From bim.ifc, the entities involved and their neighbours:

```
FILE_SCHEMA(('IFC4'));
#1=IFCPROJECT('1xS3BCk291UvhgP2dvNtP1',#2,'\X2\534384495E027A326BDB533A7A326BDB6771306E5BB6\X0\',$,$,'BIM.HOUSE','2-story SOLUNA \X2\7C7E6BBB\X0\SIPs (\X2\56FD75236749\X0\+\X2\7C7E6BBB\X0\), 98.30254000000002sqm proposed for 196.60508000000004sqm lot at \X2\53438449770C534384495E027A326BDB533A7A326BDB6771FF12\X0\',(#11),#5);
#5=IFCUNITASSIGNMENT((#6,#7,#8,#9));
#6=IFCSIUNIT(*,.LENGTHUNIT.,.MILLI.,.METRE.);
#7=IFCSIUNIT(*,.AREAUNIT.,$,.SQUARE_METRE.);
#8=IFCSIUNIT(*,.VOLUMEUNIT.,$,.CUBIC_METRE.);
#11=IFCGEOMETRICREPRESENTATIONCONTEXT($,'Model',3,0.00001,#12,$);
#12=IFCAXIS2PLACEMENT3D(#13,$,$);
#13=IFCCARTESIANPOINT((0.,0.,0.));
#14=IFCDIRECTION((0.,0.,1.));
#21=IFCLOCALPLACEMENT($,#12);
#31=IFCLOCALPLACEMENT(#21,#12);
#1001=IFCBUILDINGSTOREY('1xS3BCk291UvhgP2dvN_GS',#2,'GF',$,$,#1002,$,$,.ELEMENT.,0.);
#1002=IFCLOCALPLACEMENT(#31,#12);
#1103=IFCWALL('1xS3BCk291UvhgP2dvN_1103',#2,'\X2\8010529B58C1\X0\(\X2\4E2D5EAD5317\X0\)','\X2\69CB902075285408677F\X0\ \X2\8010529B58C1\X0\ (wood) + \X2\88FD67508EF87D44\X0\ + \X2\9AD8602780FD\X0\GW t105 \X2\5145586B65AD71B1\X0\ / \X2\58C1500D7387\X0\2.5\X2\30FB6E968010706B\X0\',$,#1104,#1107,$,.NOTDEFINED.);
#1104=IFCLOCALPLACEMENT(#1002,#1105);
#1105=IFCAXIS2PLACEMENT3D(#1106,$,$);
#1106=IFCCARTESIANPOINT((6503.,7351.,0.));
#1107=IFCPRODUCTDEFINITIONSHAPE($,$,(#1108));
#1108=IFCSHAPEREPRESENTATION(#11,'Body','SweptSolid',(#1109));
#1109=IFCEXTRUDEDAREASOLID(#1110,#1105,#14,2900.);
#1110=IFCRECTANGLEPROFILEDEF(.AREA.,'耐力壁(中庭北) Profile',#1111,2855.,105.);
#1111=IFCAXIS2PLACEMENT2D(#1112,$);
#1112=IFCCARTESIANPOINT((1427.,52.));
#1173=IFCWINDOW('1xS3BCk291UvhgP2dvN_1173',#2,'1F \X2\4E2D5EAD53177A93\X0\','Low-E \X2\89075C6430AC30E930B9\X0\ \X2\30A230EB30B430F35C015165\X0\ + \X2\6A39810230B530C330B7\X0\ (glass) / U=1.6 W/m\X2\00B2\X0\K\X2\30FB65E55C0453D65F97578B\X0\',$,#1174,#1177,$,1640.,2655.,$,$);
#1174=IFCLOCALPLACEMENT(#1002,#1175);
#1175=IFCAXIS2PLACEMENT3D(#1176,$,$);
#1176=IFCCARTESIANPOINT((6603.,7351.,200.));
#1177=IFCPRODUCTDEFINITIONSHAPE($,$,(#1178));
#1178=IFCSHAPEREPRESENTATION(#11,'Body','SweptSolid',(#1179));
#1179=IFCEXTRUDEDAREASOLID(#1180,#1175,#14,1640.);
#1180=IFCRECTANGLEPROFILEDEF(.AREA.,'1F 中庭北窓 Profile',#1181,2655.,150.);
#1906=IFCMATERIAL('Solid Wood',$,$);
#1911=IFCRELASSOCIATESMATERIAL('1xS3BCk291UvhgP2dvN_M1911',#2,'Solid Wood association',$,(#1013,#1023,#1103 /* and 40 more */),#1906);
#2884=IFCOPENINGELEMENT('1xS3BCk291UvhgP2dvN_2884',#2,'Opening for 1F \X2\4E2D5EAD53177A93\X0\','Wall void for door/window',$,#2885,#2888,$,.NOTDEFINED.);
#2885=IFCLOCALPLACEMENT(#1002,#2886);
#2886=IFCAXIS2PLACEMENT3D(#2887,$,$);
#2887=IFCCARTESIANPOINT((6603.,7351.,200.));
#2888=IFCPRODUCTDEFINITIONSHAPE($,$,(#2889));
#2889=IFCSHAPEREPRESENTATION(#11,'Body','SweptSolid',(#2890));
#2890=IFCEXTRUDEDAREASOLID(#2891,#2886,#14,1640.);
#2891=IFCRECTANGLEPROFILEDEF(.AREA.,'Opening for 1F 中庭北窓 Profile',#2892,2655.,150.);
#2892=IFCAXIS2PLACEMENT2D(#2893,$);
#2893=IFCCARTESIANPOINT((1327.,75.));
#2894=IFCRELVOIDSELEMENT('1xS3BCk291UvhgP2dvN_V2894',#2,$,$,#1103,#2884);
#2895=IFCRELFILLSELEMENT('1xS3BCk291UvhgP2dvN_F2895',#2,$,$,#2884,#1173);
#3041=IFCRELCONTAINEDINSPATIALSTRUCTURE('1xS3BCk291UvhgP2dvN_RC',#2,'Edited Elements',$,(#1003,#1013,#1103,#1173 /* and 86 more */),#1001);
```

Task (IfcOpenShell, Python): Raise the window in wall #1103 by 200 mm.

```python
import numpy as np
import ifcopenshell
import ifcopenshell.api.geometry
import ifcopenshell.util.placement
import ifcopenshell.util.unit

model = ifcopenshell.open("bim.ifc")
unit_scale = ifcopenshell.util.unit.calculate_unit_scale(model)

window = model.by_guid("1xS3BCk291UvhgP2dvN_1173")
opening = window.FillsVoids[0].RelatingOpeningElement
dz = 200.0

shift = np.array([0.0, 0.0, dz])
# The window is not placed relative to its opening, so move both.
for product in (opening, window):
    matrix = ifcopenshell.util.placement.get_local_placement(product.ObjectPlacement)
    matrix[:3, 3] += shift
    ifcopenshell.api.geometry.edit_object_placement(model, product=product, matrix=matrix, is_si=False)

print(f"moved by {dz * unit_scale:+.3f} m")

model.write("bim_updated.ifc")
```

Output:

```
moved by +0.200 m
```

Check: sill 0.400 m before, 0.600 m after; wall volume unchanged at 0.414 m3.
